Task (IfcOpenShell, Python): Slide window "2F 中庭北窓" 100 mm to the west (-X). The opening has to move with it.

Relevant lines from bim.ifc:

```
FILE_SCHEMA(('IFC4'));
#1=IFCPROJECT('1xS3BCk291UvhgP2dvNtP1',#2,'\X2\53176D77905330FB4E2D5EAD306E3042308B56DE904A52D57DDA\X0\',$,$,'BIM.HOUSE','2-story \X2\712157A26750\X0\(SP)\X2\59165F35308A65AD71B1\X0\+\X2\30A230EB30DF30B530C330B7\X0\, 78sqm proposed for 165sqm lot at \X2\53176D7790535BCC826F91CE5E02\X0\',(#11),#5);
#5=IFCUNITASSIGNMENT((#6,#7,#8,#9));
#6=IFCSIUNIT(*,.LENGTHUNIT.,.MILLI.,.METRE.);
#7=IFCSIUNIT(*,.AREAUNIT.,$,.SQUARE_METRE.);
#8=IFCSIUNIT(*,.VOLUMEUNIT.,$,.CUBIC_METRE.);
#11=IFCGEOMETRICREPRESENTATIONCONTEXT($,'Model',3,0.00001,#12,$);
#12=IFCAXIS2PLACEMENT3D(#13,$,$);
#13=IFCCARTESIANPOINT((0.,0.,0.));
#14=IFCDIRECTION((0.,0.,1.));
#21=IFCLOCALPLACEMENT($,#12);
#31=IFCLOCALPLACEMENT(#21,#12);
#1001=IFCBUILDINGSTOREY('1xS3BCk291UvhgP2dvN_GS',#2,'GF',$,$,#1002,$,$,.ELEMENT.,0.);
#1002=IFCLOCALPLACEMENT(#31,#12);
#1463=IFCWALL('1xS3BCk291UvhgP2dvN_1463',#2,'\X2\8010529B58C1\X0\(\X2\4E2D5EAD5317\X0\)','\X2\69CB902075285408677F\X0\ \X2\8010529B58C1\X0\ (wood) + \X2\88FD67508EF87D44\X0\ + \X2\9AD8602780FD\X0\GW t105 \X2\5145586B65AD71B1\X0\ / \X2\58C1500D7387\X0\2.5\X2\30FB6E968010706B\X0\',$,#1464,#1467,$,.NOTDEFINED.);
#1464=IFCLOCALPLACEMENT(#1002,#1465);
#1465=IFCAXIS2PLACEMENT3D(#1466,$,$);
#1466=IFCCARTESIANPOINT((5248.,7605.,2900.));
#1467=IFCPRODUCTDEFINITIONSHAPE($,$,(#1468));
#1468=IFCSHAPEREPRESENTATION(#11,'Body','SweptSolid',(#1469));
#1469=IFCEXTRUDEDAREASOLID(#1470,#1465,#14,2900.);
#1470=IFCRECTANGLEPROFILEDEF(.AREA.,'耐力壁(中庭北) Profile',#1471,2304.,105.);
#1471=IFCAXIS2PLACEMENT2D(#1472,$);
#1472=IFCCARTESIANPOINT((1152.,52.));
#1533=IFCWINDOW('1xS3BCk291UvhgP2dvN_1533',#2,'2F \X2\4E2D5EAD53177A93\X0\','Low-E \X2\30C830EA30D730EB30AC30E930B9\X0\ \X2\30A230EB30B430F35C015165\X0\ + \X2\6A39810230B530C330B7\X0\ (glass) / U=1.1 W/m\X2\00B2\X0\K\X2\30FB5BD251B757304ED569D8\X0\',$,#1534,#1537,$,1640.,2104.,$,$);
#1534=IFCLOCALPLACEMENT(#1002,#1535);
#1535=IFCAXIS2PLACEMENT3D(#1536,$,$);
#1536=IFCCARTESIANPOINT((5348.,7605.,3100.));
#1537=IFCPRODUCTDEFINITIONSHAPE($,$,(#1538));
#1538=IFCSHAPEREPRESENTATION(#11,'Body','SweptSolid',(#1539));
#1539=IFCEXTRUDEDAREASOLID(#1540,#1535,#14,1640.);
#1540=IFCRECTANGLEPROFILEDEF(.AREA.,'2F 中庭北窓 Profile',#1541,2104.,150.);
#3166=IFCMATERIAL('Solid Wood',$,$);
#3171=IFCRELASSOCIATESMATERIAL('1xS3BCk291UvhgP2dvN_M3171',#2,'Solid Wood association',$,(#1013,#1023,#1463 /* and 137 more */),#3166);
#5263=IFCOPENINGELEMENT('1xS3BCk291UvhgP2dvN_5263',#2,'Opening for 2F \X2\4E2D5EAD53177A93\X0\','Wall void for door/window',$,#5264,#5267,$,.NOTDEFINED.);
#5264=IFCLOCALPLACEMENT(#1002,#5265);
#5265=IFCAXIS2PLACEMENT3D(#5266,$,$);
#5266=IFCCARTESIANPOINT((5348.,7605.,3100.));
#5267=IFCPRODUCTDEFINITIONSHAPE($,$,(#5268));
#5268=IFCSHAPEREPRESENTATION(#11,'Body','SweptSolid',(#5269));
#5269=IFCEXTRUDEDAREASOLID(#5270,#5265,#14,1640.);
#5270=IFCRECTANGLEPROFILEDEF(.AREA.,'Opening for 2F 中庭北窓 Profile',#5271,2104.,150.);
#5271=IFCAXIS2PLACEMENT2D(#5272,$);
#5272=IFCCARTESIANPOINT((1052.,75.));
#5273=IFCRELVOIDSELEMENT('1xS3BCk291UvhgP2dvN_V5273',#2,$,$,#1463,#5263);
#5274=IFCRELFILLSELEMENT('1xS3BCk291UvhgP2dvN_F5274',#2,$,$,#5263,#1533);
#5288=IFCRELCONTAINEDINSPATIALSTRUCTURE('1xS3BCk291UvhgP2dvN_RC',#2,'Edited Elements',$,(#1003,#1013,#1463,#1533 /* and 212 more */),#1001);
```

```python
import ifcopenshell
import ifcopenshell.api.geometry
import ifcopenshell.util.placement
import ifcopenshell.util.unit

model = ifcopenshell.open("bim.ifc")
unit_scale = ifcopenshell.util.unit.calculate_unit_scale(model)

window = model.by_guid("1xS3BCk291UvhgP2dvN_1533")
opening = window.FillsVoids[0].RelatingOpeningElement
wall = opening.VoidsElements[0].RelatingBuildingElement

wall_matrix = ifcopenshell.util.placement.get_local_placement(wall.ObjectPlacement)
shift = wall_matrix[:3, 0] * -0.1 / unit_scale
before = ifcopenshell.util.placement.get_local_placement(window.ObjectPlacement)[:3, 3].copy()

# The window is not placed relative to its opening, so move both.
for product in (opening, window):
    matrix = ifcopenshell.util.placement.get_local_placement(product.ObjectPlacement)
    matrix[:3, 3] += shift
    ifcopenshell.api.geometry.edit_object_placement(model, product=product, matrix=matrix, is_si=False)

after = ifcopenshell.util.placement.get_local_placement(window.ObjectPlacement)[:3, 3]
print("window moved by", (after - before).round(3) + 0.0)

model.write("bim_edited.ifc")
```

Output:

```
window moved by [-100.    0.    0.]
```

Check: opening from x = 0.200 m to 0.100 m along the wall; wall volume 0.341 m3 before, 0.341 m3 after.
